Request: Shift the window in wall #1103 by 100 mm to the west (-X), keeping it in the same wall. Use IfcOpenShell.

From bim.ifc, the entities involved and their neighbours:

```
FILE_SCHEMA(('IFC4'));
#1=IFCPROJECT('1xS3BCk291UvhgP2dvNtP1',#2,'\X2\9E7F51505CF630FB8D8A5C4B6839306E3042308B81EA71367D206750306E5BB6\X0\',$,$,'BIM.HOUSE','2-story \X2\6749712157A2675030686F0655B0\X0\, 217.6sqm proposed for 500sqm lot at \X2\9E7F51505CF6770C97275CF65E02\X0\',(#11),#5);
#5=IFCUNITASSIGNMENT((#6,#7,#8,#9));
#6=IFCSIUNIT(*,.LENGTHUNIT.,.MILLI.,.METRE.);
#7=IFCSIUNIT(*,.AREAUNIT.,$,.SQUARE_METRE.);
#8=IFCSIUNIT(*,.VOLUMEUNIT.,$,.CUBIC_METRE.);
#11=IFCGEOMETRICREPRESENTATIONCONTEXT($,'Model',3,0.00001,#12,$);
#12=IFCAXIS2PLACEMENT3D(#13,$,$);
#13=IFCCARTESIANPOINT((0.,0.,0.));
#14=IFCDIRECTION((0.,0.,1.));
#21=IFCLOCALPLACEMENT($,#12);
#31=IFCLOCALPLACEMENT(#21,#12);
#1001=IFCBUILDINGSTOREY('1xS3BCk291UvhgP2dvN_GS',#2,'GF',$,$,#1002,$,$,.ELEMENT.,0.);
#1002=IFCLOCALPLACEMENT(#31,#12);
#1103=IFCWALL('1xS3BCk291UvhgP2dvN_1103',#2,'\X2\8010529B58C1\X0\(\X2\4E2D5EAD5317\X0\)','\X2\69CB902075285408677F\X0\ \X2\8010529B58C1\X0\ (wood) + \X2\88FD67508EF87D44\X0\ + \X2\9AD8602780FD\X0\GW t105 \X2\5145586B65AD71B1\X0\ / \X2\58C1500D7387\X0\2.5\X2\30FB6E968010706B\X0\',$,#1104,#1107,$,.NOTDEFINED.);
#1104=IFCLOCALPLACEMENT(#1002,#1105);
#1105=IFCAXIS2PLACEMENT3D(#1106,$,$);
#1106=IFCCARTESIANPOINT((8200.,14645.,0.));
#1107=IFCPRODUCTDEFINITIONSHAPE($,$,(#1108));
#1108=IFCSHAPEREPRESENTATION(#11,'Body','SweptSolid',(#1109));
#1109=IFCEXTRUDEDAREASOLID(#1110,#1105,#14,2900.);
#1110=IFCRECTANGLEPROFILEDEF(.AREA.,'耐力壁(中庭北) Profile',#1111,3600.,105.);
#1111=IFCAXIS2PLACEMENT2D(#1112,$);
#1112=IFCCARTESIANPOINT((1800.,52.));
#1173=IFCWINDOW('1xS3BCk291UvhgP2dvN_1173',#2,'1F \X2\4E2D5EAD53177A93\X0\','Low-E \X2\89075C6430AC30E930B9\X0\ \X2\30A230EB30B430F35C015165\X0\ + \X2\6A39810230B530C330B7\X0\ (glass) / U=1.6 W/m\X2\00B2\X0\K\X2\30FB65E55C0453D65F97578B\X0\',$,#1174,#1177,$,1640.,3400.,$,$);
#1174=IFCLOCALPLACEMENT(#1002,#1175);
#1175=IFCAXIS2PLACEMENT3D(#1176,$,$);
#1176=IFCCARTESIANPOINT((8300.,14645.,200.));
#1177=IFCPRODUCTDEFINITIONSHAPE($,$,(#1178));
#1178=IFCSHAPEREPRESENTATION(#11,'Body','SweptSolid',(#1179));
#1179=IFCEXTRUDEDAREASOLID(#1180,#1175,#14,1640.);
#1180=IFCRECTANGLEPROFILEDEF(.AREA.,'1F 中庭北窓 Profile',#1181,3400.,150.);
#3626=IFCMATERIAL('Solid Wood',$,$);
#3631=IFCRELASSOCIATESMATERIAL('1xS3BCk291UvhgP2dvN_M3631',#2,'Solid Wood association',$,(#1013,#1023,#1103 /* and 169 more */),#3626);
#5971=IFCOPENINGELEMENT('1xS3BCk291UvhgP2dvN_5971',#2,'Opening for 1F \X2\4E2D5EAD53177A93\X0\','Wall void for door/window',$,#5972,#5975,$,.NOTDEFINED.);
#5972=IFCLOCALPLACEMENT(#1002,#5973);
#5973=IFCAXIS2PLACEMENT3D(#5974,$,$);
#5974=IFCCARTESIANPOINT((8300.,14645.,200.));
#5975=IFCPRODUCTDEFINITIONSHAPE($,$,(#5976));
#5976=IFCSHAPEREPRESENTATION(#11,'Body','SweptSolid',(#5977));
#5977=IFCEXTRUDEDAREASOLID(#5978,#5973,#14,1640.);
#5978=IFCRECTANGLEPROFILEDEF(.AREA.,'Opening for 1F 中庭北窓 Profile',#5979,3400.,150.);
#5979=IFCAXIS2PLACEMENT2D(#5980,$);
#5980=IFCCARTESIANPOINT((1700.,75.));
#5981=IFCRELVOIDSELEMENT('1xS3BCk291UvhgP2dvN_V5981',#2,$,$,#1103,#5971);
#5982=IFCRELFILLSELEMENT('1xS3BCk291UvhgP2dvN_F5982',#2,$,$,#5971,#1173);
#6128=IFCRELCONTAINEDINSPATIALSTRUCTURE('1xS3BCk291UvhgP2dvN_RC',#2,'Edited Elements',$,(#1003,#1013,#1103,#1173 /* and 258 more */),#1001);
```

```python
import ifcopenshell
import ifcopenshell.api.geometry
import ifcopenshell.util.placement
import ifcopenshell.util.unit

model = ifcopenshell.open("bim.ifc")
unit_scale = ifcopenshell.util.unit.calculate_unit_scale(model)

window = model.by_guid("1xS3BCk291UvhgP2dvN_1173")
opening = window.FillsVoids[0].RelatingOpeningElement
wall = opening.VoidsElements[0].RelatingBuildingElement

wall_matrix = ifcopenshell.util.placement.get_local_placement(wall.ObjectPlacement)
shift = wall_matrix[:3, 0] * -0.1 / unit_scale
before = ifcopenshell.util.placement.get_local_placement(window.ObjectPlacement)[:3, 3].copy()

# The window is not placed relative to its opening, so move both.
for product in (opening, window):
    matrix = ifcopenshell.util.placement.get_local_placement(product.ObjectPlacement)
    matrix[:3, 3] += shift
    ifcopenshell.api.geometry.edit_object_placement(model, product=product, matrix=matrix, is_si=False)

after = ifcopenshell.util.placement.get_local_placement(window.ObjectPlacement)[:3, 3]
print("window moved by", (after - before).round(3) + 0.0)

model.write("bim_rev.ifc")
```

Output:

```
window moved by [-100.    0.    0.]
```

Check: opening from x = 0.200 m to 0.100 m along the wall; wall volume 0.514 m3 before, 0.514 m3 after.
